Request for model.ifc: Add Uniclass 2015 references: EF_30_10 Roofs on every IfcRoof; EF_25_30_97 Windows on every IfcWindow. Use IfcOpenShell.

First a look at what the model holds.

```python
import ifcopenshell

model = ifcopenshell.open("model.ifc")
print(model.schema)
print("classifications:", [c.Name for c in model.by_type("IfcClassification")])
for ifc_class in ("IfcDoor", "IfcRoof", "IfcStair", "IfcWall", "IfcWindow"):
    print(ifc_class, len(model.by_type(ifc_class)))
```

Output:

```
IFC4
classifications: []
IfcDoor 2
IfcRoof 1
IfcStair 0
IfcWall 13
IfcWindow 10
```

```python
import ifcopenshell
import ifcopenshell.api.classification

model = ifcopenshell.open("model.ifc")

system = ifcopenshell.api.classification.add_classification(model, classification="Uniclass 2015")

codes = {
    "IfcRoof": ("EF_30_10", "Roofs"),
    "IfcWindow": ("EF_25_30_97", "Windows"),
}
for ifc_class, (code, name) in codes.items():
    products = model.by_type(ifc_class)
    ifcopenshell.api.classification.add_reference(
        model, products=products, classification=system, identification=code, name=name
    )
    print(code, len(products))

model.write("model_rev.ifc")
```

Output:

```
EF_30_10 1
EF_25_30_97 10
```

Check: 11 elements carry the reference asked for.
